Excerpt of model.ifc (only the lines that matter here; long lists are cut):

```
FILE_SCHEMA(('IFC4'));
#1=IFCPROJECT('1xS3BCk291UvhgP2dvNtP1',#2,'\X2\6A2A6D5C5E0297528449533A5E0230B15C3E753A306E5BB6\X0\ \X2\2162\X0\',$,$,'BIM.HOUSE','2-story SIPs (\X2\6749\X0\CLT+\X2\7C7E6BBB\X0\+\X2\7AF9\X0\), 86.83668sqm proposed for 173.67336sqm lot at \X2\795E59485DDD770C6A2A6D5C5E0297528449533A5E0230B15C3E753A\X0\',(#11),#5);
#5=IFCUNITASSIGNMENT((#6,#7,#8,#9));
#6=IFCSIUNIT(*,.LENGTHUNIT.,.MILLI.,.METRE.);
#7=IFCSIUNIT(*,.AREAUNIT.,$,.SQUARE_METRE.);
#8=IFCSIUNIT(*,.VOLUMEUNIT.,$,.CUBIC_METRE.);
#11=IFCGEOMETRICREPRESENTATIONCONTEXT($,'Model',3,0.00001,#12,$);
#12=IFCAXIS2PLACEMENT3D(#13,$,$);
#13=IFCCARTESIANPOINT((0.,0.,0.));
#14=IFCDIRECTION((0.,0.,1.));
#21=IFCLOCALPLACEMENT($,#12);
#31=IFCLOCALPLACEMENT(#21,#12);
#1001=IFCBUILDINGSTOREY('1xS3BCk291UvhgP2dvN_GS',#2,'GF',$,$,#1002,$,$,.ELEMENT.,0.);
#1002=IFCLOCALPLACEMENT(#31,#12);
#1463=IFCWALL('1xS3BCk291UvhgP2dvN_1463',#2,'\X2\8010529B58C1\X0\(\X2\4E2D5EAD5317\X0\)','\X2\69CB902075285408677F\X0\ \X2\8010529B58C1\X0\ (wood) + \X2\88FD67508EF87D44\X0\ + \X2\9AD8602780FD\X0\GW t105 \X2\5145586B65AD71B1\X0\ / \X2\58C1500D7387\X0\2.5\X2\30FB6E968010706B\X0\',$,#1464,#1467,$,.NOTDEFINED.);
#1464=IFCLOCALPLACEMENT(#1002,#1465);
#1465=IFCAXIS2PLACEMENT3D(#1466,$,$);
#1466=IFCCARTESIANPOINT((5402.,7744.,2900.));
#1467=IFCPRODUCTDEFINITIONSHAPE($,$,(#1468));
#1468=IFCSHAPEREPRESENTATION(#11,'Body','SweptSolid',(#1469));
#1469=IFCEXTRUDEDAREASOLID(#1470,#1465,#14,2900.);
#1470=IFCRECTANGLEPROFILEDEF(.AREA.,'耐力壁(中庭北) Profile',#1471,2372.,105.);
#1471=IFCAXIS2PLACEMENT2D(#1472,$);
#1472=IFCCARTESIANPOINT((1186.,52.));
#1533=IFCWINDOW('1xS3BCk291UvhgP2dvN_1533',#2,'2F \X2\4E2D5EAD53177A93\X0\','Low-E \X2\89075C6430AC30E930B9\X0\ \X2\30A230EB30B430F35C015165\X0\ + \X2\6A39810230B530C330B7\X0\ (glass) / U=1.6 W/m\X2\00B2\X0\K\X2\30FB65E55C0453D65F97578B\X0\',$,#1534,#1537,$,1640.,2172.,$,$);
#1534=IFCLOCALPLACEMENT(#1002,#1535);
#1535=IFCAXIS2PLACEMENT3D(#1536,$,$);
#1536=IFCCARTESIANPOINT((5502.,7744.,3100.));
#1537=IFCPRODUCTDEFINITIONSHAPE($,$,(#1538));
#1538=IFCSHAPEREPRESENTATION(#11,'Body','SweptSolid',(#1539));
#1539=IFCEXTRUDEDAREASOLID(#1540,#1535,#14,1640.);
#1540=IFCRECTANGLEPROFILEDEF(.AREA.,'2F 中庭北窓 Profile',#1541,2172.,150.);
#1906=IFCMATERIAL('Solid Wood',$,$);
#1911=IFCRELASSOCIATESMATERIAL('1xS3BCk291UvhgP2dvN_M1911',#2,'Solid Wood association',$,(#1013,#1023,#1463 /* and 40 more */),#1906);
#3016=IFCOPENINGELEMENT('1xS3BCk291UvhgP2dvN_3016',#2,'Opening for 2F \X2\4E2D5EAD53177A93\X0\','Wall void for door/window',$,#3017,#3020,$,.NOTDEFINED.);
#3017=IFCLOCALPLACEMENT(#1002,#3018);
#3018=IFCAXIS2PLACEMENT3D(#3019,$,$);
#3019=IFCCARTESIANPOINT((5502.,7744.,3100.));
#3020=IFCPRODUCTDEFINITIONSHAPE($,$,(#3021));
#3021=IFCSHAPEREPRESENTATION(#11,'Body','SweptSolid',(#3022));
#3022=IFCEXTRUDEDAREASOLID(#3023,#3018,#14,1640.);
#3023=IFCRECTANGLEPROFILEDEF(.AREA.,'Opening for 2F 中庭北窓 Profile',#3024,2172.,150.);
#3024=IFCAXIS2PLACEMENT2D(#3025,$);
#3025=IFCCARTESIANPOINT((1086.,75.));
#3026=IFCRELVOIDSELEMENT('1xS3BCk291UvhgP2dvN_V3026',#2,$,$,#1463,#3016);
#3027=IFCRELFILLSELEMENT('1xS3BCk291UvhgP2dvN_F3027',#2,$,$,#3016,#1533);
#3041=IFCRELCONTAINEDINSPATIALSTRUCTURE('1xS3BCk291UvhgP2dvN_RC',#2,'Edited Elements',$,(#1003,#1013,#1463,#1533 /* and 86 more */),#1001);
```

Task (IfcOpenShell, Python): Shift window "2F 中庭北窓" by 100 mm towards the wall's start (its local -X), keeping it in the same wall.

```python
import ifcopenshell
import ifcopenshell.api.geometry
import ifcopenshell.util.placement
import ifcopenshell.util.unit

model = ifcopenshell.open("model.ifc")
unit_scale = ifcopenshell.util.unit.calculate_unit_scale(model)

window = model.by_guid("1xS3BCk291UvhgP2dvN_1533")
opening = window.FillsVoids[0].RelatingOpeningElement
wall = opening.VoidsElements[0].RelatingBuildingElement

wall_matrix = ifcopenshell.util.placement.get_local_placement(wall.ObjectPlacement)
shift = wall_matrix[:3, 0] * -0.1 / unit_scale
before = ifcopenshell.util.placement.get_local_placement(window.ObjectPlacement)[:3, 3].copy()

# The window is not placed relative to its opening, so move both.
for product in (opening, window):
    matrix = ifcopenshell.util.placement.get_local_placement(product.ObjectPlacement)
    matrix[:3, 3] += shift
    ifcopenshell.api.geometry.edit_object_placement(model, product=product, matrix=matrix, is_si=False)

after = ifcopenshell.util.placement.get_local_placement(window.ObjectPlacement)[:3, 3]
print("window moved by", (after - before).round(3) + 0.0)

model.write("model_updated.ifc")
```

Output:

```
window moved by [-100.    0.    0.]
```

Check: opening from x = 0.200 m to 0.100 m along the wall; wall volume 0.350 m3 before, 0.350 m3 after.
